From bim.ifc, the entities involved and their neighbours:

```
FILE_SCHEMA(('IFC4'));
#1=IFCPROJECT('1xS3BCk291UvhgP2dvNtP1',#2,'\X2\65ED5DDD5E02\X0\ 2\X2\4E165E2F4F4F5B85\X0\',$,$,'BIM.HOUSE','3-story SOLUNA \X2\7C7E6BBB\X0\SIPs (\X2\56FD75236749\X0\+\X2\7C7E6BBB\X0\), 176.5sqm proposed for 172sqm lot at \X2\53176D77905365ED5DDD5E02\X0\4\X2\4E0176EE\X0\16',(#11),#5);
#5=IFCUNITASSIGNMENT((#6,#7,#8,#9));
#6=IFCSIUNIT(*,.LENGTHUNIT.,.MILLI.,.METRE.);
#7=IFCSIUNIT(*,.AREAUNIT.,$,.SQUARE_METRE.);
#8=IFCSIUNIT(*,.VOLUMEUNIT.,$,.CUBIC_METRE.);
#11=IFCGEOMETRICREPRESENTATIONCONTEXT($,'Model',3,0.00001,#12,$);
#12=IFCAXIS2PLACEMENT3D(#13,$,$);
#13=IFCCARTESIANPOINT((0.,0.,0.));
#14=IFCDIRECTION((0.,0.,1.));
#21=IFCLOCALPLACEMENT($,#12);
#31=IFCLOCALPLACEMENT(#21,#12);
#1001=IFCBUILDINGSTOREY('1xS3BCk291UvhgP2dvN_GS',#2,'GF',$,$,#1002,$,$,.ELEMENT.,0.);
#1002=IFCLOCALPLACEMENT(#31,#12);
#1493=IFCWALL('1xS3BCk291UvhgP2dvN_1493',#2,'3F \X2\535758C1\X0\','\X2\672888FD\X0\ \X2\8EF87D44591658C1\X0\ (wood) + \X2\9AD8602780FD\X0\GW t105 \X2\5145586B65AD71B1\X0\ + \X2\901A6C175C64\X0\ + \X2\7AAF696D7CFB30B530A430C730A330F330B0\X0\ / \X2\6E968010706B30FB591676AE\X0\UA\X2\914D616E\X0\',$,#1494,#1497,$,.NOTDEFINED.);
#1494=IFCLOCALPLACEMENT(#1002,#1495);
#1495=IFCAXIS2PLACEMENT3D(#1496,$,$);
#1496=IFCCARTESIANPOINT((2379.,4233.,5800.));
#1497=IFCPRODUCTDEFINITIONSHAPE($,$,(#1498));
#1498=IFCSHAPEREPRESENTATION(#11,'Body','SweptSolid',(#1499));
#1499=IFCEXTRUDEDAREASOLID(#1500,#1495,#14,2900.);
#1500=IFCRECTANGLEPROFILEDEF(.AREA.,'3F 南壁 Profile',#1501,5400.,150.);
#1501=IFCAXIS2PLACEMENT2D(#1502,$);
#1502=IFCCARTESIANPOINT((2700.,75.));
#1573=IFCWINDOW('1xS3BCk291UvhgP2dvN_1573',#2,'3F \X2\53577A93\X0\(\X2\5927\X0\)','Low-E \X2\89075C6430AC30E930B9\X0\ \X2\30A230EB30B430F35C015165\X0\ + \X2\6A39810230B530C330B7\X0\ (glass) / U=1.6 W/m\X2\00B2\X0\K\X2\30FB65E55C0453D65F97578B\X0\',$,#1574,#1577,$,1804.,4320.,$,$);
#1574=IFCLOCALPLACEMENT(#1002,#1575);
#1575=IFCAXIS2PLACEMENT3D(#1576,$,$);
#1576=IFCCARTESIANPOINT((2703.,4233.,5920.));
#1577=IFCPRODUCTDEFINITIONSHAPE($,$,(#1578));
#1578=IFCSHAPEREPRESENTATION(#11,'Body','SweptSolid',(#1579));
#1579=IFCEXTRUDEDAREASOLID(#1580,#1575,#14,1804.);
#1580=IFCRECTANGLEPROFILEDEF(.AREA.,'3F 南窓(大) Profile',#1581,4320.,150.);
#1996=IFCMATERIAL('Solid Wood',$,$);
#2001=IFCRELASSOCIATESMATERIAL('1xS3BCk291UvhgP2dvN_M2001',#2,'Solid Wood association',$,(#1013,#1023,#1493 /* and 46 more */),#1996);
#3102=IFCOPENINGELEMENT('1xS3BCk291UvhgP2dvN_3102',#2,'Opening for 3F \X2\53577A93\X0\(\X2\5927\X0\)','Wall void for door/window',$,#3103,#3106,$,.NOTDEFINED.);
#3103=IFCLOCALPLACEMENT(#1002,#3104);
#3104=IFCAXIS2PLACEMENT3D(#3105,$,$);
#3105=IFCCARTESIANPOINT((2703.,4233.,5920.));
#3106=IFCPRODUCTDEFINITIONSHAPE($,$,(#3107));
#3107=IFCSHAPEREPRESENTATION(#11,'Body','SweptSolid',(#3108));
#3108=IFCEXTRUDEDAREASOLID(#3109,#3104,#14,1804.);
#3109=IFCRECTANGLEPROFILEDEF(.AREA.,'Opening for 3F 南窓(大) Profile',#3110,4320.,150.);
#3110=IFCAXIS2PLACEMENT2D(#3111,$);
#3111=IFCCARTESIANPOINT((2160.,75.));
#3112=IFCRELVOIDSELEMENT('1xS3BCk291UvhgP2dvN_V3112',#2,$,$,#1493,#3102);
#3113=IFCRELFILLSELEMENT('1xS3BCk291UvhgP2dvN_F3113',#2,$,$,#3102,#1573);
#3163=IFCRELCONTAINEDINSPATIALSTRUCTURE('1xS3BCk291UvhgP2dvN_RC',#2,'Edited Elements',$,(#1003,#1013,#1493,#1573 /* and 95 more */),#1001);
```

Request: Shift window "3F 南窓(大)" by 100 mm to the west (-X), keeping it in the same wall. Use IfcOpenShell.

```python
import ifcopenshell
import ifcopenshell.api.geometry
import ifcopenshell.util.placement

model = ifcopenshell.open("bim.ifc")

window = model.by_guid("1xS3BCk291UvhgP2dvN_1573")
opening = window.FillsVoids[0].RelatingOpeningElement
wall = opening.VoidsElements[0].RelatingBuildingElement

wall_matrix = ifcopenshell.util.placement.get_local_placement(wall.ObjectPlacement)
shift = wall_matrix[:3, 0] * -100.0
before = ifcopenshell.util.placement.get_local_placement(window.ObjectPlacement)[:3, 3].copy()

# The window is not placed relative to its opening, so move both.
for product in (opening, window):
    matrix = ifcopenshell.util.placement.get_local_placement(product.ObjectPlacement)
    matrix[:3, 3] += shift
    ifcopenshell.api.geometry.edit_object_placement(model, product=product, matrix=matrix, is_si=False)

after = ifcopenshell.util.placement.get_local_placement(window.ObjectPlacement)[:3, 3]
print("window moved by", (after - before).round(3) + 0.0)

model.write("bim-out.ifc")
```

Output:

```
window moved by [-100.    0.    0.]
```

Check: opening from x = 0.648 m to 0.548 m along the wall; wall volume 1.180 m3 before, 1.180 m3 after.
